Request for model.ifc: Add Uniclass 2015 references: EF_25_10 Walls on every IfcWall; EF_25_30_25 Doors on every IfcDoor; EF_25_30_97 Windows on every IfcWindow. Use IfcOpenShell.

First a look at what the model holds.

```python
import ifcopenshell

model = ifcopenshell.open("model.ifc")
print(model.schema)
print("classifications:", [c.Name for c in model.by_type("IfcClassification")])
for ifc_class in ("IfcDoor", "IfcRoof", "IfcStair", "IfcWall", "IfcWindow"):
    print(ifc_class, len(model.by_type(ifc_class)))
```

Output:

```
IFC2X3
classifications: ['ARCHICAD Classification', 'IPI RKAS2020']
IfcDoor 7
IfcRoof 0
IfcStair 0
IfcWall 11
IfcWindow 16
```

```python
import ifcopenshell
import ifcopenshell.api.classification

model = ifcopenshell.open("model.ifc")

# IFC2X3 requires Source and Edition and has no link from the project to the system.
system = model.create_entity("IfcClassification", Source="NBS", Edition="2015", Name="Uniclass 2015")

codes = {
    "IfcWall": ("EF_25_10", "Walls"),
    "IfcDoor": ("EF_25_30_25", "Doors"),
    "IfcWindow": ("EF_25_30_97", "Windows"),
}
for ifc_class, (code, name) in codes.items():
    products = model.by_type(ifc_class)
    ifcopenshell.api.classification.add_reference(
        model, products=products, classification=system, identification=code, name=name
    )
    print(code, len(products))

model.write("model_v2.ifc")
```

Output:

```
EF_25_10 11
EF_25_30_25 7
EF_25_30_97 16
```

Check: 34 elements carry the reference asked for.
